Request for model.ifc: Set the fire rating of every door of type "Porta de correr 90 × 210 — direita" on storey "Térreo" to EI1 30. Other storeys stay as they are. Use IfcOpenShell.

First a look at what the model holds.

```python
import ifcopenshell
import ifcopenshell.util.element

model = ifcopenshell.open("model.ifc")
print(model.schema)
storey = next(s for s in model.by_type("IfcBuildingStorey") if s.Name == "Térreo")
doors = [e for e in ifcopenshell.util.element.get_decomposition(storey) if e.is_a("IfcDoor")]
seen = {}
for e in doors:
    element_type = ifcopenshell.util.element.get_type(e)
    key = (element_type.Name if element_type != e and element_type else None, ifcopenshell.util.element.get_pset(e, "Pset_DoorCommon", "FireRating"))
    seen[key] = seen.get(key, 0) + 1
for (name, value), count in sorted(seen.items(), key=str):
    print(count, "x", name, "|", value)
```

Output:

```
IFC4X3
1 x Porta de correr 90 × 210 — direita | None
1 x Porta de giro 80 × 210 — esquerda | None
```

```python
import ifcopenshell
import ifcopenshell.api.pset
import ifcopenshell.util.element

model = ifcopenshell.open("model.ifc")

storey = next(s for s in model.by_type("IfcBuildingStorey") if s.Name == "Térreo")
doors = [e for e in ifcopenshell.util.element.get_decomposition(storey) if e.is_a("IfcDoor")]

count = 0
for e in doors:
    element_type = ifcopenshell.util.element.get_type(e)
    if element_type in (None, e) or element_type.Name != "Porta de correr 90 × 210 — direita":
        continue
    # add_pset returns the element's existing set when there is one.
    pset = ifcopenshell.api.pset.add_pset(model, product=e, name="Pset_DoorCommon")
    ifcopenshell.api.pset.edit_pset(model, pset=pset, properties={"FireRating": "EI1 30"})
    count += 1

print(count, "doors updated")

model.write("model_v2.ifc")
```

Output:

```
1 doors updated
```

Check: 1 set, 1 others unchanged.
